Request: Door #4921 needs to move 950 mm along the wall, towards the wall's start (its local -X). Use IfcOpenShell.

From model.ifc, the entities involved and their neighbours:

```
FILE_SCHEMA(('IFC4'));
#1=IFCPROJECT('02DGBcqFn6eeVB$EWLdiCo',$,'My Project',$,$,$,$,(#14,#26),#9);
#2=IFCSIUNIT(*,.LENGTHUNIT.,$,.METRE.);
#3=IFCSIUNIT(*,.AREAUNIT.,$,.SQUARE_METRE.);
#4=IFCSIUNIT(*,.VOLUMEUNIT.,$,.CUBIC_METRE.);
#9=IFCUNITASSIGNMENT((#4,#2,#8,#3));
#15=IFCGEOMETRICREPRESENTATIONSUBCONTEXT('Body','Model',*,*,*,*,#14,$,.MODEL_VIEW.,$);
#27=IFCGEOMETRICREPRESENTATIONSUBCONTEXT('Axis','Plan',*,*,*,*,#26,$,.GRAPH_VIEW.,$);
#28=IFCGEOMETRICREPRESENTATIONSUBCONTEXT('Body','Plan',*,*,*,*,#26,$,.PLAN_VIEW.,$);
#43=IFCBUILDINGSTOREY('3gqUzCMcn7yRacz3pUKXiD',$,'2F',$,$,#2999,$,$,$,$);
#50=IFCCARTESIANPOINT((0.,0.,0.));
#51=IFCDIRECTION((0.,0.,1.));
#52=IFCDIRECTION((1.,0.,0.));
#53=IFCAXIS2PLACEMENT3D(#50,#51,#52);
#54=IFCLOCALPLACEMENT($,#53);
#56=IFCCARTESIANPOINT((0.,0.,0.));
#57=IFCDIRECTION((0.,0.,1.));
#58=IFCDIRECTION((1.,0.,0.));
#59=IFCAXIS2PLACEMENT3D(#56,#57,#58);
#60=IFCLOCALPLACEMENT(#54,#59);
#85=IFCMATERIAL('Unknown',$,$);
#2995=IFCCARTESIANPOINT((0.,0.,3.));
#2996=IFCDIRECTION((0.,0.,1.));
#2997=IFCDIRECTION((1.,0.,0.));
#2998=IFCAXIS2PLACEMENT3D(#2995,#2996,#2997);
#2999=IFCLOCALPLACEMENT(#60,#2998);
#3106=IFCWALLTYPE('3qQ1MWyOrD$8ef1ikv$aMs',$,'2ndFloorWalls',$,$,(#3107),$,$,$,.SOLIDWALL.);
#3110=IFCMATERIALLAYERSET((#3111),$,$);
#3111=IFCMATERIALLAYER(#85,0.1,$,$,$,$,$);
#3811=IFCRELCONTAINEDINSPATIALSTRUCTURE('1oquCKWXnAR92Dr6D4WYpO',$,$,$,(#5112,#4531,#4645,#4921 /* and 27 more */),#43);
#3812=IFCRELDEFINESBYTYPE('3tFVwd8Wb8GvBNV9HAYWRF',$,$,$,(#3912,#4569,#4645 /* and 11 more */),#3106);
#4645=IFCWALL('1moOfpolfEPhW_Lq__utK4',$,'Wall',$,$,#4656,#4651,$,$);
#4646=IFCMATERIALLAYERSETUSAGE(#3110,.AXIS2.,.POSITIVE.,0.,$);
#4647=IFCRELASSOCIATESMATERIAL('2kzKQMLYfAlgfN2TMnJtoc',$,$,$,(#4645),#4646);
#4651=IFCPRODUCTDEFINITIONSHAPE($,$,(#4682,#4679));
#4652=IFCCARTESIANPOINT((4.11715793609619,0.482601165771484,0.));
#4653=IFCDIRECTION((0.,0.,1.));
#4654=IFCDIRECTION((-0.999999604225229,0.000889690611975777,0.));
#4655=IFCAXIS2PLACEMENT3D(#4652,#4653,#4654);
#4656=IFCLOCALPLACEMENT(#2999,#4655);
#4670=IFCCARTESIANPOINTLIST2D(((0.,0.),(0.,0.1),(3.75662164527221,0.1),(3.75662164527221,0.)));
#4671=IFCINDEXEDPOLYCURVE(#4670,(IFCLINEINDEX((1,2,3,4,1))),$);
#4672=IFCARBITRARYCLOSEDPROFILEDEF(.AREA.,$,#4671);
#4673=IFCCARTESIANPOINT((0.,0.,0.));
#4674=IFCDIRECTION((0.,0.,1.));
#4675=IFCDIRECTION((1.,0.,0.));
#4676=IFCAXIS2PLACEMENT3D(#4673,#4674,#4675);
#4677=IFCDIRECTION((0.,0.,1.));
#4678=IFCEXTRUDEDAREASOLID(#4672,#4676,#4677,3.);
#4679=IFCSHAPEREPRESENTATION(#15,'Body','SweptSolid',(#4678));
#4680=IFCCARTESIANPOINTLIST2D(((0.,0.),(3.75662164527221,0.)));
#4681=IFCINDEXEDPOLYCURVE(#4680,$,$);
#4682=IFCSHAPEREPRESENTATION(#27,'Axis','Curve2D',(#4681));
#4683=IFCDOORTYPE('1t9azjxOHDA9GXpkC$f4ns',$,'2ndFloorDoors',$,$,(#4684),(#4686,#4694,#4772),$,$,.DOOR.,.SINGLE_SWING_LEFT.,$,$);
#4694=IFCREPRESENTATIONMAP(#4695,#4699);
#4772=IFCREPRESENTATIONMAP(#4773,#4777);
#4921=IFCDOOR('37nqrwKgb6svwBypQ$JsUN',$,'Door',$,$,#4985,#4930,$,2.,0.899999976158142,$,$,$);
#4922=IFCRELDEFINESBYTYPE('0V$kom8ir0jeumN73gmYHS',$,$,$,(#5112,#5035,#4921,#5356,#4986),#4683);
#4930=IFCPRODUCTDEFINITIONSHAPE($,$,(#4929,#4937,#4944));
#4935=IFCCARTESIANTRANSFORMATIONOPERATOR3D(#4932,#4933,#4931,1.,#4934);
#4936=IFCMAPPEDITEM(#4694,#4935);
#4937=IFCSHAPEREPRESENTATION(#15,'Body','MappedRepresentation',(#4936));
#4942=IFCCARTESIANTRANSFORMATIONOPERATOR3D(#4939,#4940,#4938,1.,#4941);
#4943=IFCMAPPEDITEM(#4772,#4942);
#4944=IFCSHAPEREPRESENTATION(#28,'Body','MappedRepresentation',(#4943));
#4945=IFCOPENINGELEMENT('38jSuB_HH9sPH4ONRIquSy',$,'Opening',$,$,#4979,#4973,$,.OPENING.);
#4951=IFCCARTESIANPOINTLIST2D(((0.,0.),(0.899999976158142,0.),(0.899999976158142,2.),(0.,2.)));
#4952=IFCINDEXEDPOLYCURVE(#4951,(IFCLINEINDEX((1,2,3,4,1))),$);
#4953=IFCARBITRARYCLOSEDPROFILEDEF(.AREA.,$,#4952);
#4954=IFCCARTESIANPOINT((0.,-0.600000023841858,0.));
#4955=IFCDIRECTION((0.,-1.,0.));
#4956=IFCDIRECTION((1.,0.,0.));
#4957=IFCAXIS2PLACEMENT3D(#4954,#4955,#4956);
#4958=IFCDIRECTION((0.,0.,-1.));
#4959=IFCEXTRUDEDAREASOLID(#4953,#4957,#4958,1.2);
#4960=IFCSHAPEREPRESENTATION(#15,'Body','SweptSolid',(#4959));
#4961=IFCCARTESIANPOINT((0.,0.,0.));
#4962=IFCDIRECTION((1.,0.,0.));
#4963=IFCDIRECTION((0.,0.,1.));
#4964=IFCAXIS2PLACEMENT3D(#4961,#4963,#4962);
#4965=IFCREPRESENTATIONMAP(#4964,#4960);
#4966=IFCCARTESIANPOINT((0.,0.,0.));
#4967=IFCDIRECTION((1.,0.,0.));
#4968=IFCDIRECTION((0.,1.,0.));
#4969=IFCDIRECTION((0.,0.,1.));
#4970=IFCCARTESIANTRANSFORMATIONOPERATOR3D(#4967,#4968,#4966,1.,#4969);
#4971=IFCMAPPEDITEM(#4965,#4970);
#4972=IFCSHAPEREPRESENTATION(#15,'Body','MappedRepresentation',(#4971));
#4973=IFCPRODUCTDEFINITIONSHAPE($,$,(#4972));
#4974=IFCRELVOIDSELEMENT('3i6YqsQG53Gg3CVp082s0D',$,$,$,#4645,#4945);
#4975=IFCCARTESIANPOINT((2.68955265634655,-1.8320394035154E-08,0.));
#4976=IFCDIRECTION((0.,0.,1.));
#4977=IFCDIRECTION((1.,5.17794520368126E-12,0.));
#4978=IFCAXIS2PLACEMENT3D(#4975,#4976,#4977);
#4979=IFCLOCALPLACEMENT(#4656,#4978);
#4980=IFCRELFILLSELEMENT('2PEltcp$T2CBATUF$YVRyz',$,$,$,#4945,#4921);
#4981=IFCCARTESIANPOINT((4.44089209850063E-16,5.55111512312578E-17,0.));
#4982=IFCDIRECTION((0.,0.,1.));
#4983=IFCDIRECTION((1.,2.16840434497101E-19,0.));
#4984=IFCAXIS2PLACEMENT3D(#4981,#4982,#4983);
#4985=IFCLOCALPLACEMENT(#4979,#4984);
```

```python
import ifcopenshell
import ifcopenshell.api.geometry
import ifcopenshell.util.placement

model = ifcopenshell.open("model.ifc")

door = model.by_guid("37nqrwKgb6svwBypQ$JsUN")
opening = door.FillsVoids[0].RelatingOpeningElement
wall = opening.VoidsElements[0].RelatingBuildingElement

wall_matrix = ifcopenshell.util.placement.get_local_placement(wall.ObjectPlacement)
shift = wall_matrix[:3, 0] * -0.95
before = ifcopenshell.util.placement.get_local_placement(door.ObjectPlacement)[:3, 3].copy()

# The door is placed relative to its opening, so it follows when the opening moves.
matrix = ifcopenshell.util.placement.get_local_placement(opening.ObjectPlacement)
matrix[:3, 3] += shift
ifcopenshell.api.geometry.edit_object_placement(
    model, product=opening, matrix=matrix, is_si=False, should_transform_children=True
)

after = ifcopenshell.util.placement.get_local_placement(door.ObjectPlacement)[:3, 3]
print("door moved by", (after - before).round(3) + 0.0)

model.write("model-out.ifc")
```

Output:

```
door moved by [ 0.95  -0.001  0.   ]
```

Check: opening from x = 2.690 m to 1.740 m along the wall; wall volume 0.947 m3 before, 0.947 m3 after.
